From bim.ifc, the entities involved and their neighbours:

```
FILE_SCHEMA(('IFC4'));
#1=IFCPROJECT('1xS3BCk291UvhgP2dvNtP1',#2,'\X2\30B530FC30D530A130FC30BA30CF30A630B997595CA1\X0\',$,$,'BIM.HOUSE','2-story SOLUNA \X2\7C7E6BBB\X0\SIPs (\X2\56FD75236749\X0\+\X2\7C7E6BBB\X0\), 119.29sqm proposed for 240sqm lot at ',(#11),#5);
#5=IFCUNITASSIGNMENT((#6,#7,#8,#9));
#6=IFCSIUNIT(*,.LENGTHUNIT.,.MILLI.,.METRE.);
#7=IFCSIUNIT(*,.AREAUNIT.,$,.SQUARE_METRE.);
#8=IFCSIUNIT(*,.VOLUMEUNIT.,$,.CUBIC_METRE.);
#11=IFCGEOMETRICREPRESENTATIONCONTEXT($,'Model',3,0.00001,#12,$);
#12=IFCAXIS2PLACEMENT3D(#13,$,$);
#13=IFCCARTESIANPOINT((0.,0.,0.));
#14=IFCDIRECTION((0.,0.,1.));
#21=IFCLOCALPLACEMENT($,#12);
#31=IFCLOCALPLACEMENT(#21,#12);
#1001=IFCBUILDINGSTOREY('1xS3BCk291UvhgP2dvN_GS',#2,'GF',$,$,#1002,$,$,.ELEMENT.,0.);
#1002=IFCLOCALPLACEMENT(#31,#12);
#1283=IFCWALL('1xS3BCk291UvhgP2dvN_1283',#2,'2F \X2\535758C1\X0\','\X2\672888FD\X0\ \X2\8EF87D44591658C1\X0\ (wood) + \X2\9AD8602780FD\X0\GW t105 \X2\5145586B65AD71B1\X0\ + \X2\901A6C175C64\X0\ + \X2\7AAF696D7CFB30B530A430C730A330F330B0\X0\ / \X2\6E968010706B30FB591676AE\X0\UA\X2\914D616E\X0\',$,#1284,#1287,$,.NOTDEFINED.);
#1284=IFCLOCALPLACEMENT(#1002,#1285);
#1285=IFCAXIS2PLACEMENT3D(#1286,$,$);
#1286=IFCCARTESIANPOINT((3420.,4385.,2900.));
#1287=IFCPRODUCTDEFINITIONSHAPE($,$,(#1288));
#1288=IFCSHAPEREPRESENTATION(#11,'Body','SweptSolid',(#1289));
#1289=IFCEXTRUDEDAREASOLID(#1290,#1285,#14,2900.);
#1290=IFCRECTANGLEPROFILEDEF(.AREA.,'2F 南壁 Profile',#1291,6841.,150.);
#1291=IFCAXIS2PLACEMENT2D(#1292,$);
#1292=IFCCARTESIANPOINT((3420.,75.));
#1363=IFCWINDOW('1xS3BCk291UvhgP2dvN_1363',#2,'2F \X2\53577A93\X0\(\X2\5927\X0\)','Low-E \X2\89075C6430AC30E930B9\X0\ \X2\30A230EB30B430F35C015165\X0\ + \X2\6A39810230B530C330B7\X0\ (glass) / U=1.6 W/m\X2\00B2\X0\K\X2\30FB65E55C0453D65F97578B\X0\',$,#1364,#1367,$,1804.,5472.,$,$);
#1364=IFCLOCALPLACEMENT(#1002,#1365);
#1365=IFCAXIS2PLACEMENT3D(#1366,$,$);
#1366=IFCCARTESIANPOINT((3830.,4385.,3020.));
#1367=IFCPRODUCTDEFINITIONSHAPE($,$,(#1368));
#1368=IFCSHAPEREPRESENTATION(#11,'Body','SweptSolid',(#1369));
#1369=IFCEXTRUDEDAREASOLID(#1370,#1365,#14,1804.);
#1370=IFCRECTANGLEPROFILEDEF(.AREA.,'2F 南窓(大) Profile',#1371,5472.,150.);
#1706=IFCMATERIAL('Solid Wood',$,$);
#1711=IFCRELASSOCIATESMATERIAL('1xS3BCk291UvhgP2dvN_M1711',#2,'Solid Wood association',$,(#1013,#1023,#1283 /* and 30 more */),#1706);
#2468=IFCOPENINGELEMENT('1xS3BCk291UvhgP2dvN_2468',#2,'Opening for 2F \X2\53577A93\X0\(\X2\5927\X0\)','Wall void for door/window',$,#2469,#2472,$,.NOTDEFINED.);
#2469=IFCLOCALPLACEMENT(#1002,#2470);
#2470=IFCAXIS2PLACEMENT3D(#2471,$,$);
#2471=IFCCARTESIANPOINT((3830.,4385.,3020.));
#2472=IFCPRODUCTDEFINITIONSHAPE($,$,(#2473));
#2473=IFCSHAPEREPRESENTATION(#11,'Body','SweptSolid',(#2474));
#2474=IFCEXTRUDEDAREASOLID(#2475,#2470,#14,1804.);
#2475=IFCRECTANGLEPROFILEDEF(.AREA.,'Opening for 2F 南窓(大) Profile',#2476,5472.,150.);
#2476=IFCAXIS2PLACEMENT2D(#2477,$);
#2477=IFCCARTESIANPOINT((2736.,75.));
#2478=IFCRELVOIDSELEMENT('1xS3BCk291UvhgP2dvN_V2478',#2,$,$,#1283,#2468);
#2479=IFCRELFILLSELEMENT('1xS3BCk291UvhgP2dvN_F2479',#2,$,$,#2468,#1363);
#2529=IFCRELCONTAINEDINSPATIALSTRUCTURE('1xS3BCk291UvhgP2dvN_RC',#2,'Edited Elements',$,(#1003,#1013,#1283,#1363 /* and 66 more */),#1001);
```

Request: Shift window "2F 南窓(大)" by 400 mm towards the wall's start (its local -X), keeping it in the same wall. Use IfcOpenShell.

```python
import ifcopenshell
import ifcopenshell.api.geometry
import ifcopenshell.util.placement

model = ifcopenshell.open("bim.ifc")

window = model.by_id(1363)
opening = window.FillsVoids[0].RelatingOpeningElement
wall = opening.VoidsElements[0].RelatingBuildingElement

wall_matrix = ifcopenshell.util.placement.get_local_placement(wall.ObjectPlacement)
shift = wall_matrix[:3, 0] * -400.0
before = ifcopenshell.util.placement.get_local_placement(window.ObjectPlacement)[:3, 3].copy()

# The window is not placed relative to its opening, so move both.
for product in (opening, window):
    matrix = ifcopenshell.util.placement.get_local_placement(product.ObjectPlacement)
    matrix[:3, 3] += shift
    ifcopenshell.api.geometry.edit_object_placement(model, product=product, matrix=matrix, is_si=False)

after = ifcopenshell.util.placement.get_local_placement(window.ObjectPlacement)[:3, 3]
print("window moved by", (after - before).round(3) + 0.0)

model.write("bim_rev.ifc")
```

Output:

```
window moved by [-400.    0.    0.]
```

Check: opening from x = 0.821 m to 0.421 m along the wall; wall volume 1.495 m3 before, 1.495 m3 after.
